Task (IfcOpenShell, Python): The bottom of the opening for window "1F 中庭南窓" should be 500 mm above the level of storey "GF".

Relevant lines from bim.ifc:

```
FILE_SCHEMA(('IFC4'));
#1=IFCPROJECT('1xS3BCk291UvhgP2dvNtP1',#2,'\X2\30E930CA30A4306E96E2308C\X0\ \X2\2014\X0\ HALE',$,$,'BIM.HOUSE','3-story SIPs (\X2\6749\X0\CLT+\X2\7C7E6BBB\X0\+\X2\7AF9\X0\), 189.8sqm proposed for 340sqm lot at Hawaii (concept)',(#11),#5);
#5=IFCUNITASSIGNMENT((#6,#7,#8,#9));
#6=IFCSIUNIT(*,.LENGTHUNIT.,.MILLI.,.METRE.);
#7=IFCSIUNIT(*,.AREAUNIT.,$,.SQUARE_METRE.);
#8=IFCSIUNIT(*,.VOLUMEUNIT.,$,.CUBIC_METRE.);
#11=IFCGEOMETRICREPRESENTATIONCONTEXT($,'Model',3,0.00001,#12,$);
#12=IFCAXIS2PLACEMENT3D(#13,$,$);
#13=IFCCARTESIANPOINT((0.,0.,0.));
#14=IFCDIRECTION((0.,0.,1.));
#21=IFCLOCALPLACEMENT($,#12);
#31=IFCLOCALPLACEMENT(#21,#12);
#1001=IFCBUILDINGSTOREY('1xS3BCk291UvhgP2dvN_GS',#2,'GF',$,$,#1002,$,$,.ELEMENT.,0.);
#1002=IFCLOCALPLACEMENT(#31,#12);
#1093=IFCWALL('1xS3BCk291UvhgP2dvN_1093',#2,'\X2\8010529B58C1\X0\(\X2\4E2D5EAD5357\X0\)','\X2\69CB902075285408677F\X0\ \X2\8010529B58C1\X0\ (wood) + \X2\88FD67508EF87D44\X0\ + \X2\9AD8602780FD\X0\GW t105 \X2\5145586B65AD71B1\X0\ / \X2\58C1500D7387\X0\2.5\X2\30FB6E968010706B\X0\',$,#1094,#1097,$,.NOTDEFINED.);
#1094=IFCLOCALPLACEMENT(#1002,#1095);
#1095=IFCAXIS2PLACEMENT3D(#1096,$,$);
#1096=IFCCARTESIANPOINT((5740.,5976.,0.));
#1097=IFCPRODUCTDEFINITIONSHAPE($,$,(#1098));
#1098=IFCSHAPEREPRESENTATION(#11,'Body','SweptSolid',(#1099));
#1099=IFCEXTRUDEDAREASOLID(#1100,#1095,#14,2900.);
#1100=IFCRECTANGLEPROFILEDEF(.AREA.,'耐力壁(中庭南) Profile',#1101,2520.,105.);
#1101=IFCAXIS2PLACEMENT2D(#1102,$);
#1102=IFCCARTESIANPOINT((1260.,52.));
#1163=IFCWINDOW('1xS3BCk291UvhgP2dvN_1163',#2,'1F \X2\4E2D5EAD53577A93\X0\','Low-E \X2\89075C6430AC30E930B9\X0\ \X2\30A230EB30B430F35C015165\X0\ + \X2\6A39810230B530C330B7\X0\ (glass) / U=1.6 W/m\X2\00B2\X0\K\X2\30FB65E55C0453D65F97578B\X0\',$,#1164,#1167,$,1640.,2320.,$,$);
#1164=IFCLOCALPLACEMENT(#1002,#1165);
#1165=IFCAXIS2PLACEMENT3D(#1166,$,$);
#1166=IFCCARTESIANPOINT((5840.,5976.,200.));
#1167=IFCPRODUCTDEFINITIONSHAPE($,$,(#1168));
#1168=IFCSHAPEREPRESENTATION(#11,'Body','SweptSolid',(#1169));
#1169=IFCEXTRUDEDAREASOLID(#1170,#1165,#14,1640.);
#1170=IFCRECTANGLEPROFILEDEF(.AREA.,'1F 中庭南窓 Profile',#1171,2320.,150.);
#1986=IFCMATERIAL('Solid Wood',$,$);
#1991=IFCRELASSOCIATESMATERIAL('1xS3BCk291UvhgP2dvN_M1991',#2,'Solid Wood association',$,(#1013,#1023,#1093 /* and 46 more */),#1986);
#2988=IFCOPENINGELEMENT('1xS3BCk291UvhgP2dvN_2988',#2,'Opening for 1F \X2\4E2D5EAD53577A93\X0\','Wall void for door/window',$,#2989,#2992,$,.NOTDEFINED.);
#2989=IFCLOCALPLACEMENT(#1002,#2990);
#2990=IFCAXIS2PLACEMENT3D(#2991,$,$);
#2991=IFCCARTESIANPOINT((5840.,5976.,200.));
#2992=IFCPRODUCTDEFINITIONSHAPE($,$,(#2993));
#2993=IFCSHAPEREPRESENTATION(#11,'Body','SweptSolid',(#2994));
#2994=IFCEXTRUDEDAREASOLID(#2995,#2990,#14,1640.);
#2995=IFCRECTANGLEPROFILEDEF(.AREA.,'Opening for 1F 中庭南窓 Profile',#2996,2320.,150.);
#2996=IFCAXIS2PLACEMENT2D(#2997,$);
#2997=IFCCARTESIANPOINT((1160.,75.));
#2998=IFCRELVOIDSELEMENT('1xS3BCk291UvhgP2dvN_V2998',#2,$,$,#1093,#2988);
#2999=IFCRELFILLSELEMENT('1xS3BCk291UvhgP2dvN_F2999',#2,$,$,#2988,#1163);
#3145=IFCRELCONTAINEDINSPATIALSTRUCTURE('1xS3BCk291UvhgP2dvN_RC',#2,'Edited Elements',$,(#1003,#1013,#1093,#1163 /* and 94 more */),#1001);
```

```python
import numpy as np
import ifcopenshell
import ifcopenshell.api.geometry
import ifcopenshell.geom
import ifcopenshell.util.element
import ifcopenshell.util.placement
import ifcopenshell.util.shape
import ifcopenshell.util.unit

model = ifcopenshell.open("bim.ifc")
unit_scale = ifcopenshell.util.unit.calculate_unit_scale(model)

window = model.by_guid("1xS3BCk291UvhgP2dvN_1163")
opening = window.FillsVoids[0].RelatingOpeningElement
storey = ifcopenshell.util.element.get_container(window, ifc_class="IfcBuildingStorey")
level = ifcopenshell.util.placement.get_local_placement(storey.ObjectPlacement)[2, 3]

# The opening's origin need not be at the sill, so measure its lowest point.
shape = ifcopenshell.geom.create_shape(ifcopenshell.geom.settings(), opening)
bottom = ifcopenshell.util.shape.get_shape_bottom_elevation(shape, shape.geometry) / unit_scale
dz = level + 0.5 / unit_scale - bottom

shift = np.array([0.0, 0.0, dz])
# The window is not placed relative to its opening, so move both.
for product in (opening, window):
    matrix = ifcopenshell.util.placement.get_local_placement(product.ObjectPlacement)
    matrix[:3, 3] += shift
    ifcopenshell.api.geometry.edit_object_placement(model, product=product, matrix=matrix, is_si=False)

print(f"moved by {dz * unit_scale:+.3f} m")

model.write("bim_edited.ifc")
```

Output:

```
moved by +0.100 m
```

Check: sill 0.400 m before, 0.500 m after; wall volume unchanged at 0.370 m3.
